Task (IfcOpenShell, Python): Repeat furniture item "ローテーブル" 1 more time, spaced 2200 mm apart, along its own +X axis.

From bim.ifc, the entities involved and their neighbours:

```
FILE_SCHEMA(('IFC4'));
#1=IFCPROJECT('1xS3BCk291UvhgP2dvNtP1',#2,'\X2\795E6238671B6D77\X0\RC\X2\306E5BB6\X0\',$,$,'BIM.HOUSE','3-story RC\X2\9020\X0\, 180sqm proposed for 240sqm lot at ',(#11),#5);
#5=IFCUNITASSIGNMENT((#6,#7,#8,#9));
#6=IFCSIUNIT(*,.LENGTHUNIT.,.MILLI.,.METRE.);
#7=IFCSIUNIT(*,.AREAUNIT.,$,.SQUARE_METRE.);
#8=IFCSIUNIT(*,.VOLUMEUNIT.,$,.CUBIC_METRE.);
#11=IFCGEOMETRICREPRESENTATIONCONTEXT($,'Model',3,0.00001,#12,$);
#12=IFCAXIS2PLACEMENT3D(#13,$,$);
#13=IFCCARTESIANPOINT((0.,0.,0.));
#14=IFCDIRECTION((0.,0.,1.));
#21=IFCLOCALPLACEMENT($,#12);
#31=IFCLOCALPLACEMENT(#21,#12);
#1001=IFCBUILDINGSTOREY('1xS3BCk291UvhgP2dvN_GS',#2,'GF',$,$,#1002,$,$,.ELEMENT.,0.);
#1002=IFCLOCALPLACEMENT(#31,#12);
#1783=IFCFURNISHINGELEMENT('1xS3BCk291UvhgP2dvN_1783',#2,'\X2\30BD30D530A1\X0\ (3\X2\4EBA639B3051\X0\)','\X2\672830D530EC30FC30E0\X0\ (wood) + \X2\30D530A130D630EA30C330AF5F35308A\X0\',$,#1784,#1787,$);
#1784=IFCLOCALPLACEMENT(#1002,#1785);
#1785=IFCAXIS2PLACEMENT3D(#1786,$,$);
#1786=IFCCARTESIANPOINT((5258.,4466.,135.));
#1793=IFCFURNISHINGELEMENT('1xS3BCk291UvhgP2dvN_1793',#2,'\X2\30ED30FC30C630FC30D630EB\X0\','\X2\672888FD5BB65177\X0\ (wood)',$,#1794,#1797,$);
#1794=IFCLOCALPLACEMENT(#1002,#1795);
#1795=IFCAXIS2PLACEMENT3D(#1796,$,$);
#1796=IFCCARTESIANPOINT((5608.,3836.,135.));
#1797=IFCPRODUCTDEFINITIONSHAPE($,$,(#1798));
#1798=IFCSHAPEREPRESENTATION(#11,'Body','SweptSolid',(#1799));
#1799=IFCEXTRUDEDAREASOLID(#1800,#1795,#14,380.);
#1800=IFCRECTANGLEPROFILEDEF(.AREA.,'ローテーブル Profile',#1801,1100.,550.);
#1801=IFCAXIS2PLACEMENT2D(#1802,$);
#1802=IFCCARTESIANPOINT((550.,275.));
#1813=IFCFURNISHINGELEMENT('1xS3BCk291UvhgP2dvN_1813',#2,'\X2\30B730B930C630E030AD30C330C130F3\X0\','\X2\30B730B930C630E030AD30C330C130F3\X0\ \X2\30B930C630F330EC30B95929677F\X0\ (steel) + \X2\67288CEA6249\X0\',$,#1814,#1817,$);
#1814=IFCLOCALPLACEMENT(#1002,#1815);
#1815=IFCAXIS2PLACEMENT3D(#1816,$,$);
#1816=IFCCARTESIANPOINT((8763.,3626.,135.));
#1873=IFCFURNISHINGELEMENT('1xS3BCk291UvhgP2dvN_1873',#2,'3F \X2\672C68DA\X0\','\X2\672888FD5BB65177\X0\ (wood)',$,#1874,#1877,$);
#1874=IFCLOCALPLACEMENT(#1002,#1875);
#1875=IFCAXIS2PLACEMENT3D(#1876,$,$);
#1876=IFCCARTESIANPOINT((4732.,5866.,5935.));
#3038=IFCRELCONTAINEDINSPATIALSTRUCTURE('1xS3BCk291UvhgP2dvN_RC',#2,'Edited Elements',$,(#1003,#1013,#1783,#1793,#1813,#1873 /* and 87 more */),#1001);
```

```python
import ifcopenshell
import ifcopenshell.api.geometry
import ifcopenshell.api.root
import ifcopenshell.util.element
import ifcopenshell.util.placement

model = ifcopenshell.open("bim.ifc")


def reuse_history(source, copy):
    """copy_class also copies each property set's owner history, people and application; keep the originals."""
    for rel in copy.IsDefinedBy:
        if rel.is_a("IfcRelDefinesByProperties") and (history := rel.RelatingPropertyDefinition.OwnerHistory):
            rel.RelatingPropertyDefinition.OwnerHistory = source.OwnerHistory
            ifcopenshell.util.element.remove_deep2(model, history)


source = model.by_id(1793)
base = ifcopenshell.util.placement.get_local_placement(source.ObjectPlacement)
step = base[:3, 0] * 2200.0

for i in range(1, 2):
    copy = ifcopenshell.api.root.copy_class(model, product=source)
    copy.Representation = ifcopenshell.util.element.copy_deep(
        model, source.Representation, exclude=["IfcGeometricRepresentationContext", "IfcRepresentationMap"]
    )
    reuse_history(source, copy)
    matrix = base.copy()
    matrix[:3, 3] += i * step
    print("added at", matrix[:3, 3].round(3) + 0.0)
    ifcopenshell.api.geometry.edit_object_placement(model, product=copy, matrix=matrix, is_si=False)

model.write("bim-out.ifc")
```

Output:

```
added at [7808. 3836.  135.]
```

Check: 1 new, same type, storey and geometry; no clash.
